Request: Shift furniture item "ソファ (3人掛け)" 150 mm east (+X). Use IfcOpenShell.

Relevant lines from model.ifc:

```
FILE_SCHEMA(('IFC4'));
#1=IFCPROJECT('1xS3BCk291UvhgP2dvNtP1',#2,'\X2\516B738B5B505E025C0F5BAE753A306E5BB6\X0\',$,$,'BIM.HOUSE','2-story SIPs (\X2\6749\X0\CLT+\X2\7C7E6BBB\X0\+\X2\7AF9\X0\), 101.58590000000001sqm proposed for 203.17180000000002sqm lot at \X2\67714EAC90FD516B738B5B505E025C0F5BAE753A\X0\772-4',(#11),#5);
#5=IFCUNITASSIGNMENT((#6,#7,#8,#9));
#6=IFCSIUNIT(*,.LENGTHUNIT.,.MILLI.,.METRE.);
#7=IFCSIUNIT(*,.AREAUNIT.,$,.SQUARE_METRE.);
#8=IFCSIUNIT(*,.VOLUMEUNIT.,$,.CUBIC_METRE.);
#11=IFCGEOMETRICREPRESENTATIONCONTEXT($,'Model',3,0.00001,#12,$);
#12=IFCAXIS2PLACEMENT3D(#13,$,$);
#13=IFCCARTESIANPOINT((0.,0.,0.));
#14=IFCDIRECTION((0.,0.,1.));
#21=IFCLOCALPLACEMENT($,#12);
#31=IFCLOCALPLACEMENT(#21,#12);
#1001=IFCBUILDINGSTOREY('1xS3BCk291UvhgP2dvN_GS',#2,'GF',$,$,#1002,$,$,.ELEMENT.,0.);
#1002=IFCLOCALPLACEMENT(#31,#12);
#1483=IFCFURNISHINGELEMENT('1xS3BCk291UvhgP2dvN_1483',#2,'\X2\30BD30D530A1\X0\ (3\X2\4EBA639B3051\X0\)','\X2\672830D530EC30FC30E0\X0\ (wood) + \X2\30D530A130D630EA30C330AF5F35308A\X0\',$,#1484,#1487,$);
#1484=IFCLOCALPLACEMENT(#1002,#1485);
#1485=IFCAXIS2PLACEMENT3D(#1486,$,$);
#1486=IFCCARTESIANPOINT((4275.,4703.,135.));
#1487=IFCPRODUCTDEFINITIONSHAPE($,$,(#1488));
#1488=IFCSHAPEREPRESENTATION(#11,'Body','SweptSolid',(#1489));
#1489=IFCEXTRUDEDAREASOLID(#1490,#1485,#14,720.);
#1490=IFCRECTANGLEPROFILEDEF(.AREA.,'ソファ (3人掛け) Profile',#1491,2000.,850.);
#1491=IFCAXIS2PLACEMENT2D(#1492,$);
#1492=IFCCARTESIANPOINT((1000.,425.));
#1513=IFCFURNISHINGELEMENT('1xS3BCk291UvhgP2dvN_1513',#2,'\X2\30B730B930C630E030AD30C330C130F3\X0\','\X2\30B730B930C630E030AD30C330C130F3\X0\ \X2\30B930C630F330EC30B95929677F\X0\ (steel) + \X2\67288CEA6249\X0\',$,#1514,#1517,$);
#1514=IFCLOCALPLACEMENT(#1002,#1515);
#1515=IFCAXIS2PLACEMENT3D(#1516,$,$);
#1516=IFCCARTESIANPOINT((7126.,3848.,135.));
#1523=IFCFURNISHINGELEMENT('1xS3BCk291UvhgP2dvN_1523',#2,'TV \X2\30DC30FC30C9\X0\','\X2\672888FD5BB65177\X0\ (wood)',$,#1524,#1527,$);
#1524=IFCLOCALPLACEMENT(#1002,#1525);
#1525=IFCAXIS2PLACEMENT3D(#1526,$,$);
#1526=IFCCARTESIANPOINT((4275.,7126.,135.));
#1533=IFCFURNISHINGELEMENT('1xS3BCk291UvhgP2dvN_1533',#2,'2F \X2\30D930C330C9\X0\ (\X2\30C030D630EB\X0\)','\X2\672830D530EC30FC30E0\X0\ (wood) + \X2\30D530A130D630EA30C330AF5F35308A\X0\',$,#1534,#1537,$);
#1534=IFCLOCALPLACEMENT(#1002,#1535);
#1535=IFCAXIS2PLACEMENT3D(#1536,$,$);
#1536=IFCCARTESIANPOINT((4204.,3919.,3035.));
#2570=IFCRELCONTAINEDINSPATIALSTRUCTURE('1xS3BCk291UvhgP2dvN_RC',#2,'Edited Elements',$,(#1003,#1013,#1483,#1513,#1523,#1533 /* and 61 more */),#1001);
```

```python
import ifcopenshell
import ifcopenshell.api.geometry
import ifcopenshell.util.placement
import ifcopenshell.util.unit

model = ifcopenshell.open("model.ifc")
unit_scale = ifcopenshell.util.unit.calculate_unit_scale(model)

item = model.by_guid("1xS3BCk291UvhgP2dvN_1483")
matrix = ifcopenshell.util.placement.get_local_placement(item.ObjectPlacement)
matrix[0, 3] += 0.15 / unit_scale
ifcopenshell.api.geometry.edit_object_placement(model, product=item, matrix=matrix, is_si=False)

print(ifcopenshell.util.placement.get_local_placement(item.ObjectPlacement).round(3) + 0.0)

model.write("model_updated.ifc")
```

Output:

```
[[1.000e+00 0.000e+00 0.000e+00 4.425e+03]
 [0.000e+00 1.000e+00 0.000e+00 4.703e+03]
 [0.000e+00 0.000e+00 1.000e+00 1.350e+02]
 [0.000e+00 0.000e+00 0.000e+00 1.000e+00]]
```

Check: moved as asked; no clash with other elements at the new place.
